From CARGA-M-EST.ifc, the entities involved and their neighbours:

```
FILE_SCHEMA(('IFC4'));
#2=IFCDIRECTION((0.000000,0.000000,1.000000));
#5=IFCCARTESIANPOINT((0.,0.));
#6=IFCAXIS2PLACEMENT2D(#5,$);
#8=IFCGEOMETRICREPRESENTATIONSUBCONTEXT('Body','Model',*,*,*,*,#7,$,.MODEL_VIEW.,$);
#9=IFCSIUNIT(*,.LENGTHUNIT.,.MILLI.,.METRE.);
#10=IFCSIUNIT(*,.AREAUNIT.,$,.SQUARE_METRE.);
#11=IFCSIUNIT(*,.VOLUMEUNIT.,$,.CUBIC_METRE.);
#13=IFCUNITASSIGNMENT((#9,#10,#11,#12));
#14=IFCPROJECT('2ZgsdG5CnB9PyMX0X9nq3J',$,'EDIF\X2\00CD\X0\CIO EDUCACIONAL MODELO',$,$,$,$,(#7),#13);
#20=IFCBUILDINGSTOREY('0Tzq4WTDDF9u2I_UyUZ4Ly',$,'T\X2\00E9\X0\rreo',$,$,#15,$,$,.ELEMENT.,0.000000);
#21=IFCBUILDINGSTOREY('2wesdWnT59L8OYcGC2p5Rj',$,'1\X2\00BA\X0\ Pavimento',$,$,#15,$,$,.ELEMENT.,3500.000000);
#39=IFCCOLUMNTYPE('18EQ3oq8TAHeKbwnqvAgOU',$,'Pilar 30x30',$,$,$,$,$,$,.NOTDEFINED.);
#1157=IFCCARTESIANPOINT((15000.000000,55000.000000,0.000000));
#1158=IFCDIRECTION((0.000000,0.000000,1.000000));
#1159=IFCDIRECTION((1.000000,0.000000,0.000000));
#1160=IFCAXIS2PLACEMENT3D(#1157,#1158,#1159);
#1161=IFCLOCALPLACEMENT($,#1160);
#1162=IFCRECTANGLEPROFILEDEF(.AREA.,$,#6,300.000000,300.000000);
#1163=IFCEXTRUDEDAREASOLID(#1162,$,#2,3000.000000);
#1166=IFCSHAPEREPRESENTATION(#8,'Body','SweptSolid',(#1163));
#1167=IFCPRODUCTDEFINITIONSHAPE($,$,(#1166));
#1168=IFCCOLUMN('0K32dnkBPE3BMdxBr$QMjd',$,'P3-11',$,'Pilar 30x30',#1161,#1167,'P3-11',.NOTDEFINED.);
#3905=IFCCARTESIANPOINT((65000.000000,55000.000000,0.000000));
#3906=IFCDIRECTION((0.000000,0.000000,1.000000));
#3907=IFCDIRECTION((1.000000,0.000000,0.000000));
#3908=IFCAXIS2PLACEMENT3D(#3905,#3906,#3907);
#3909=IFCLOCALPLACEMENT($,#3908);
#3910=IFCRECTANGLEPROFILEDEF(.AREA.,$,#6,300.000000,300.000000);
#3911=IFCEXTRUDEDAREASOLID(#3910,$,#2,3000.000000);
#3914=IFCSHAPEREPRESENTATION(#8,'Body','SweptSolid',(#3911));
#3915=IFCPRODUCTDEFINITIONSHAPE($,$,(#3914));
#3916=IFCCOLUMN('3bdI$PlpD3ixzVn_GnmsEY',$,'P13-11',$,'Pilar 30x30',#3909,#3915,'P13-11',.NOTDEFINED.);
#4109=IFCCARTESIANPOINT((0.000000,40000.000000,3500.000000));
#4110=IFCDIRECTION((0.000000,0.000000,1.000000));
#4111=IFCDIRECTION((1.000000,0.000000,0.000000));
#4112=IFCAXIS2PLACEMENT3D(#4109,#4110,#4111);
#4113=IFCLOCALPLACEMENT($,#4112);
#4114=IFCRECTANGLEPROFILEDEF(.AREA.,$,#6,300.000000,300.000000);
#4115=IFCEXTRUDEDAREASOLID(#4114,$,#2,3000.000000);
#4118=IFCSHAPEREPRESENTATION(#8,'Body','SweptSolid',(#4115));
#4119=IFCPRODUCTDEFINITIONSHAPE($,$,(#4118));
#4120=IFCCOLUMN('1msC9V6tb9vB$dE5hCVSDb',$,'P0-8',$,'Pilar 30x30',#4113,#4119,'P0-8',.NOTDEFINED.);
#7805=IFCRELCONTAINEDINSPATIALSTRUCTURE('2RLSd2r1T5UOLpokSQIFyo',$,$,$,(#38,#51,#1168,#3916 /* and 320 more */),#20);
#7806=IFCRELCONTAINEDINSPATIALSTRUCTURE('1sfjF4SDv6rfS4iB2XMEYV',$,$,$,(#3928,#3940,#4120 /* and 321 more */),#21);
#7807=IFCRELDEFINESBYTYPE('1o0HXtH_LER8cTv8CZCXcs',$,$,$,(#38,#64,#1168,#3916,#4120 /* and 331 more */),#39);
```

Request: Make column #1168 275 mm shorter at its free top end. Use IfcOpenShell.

```python
import ifcopenshell
import ifcopenshell.util.representation
import ifcopenshell.util.unit

model = ifcopenshell.open("CARGA-M-EST.ifc")
unit_scale = ifcopenshell.util.unit.calculate_unit_scale(model)

member = model.by_guid("0K32dnkBPE3BMdxBr$QMjd")
change = -0.275 / unit_scale

# The extrusion runs towards the end named, so only its depth changes.
body = ifcopenshell.util.representation.get_representation(member, "Model", "Body")
solid = body.Items[0]
old_length = solid.Depth
solid.Depth += change

print(f"length {old_length:g} -> {solid.Depth:g}")

model.write("CARGA-M-EST-out.ifc")
```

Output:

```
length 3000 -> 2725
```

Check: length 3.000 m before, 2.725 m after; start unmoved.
